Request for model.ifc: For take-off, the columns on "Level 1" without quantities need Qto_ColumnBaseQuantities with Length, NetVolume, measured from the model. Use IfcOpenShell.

First a look at what the model holds.

```python
import ifcopenshell
import ifcopenshell.util.element
import ifcopenshell.util.unit

model = ifcopenshell.open("model.ifc")
print(model.schema)
for unit_type in ("LENGTHUNIT", "AREAUNIT", "VOLUMEUNIT"):
    print(unit_type, ifcopenshell.util.unit.calculate_unit_scale(model, unit_type))
storey = next(s for s in model.by_type("IfcBuildingStorey") if s.Name == "Level 1")
columns = [e for e in ifcopenshell.util.element.get_decomposition(storey) if e.is_a("IfcColumn")]
for e in sorted(columns, key=lambda e: e.id()):
    print(e.id(), e.is_a(), e.Name, list(ifcopenshell.util.element.get_psets(e, qtos_only=True)), sep=" | ")
```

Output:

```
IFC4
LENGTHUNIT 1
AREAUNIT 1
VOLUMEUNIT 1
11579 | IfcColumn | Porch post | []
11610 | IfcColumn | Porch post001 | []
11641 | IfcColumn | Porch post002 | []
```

```python
import ifcopenshell
import ifcopenshell.api.pset
import ifcopenshell.geom
import ifcopenshell.util.element
import ifcopenshell.util.shape
import ifcopenshell.util.unit

model = ifcopenshell.open("model.ifc")
unit_scale = ifcopenshell.util.unit.calculate_unit_scale(model)
volume_scale = ifcopenshell.util.unit.calculate_unit_scale(model, "VOLUMEUNIT")
settings = ifcopenshell.geom.settings()

storey = next(s for s in model.by_type("IfcBuildingStorey") if s.Name == "Level 1")
columns = [e for e in ifcopenshell.util.element.get_decomposition(storey) if e.is_a("IfcColumn")]

for e in sorted(columns, key=lambda e: e.id()):
    if ifcopenshell.util.element.get_psets(e, qtos_only=True, should_inherit=False):
        continue
    # Geometry comes back in metres, in the element's own axes.
    shape = ifcopenshell.geom.create_shape(settings, e)
    values = {
        "Length": ifcopenshell.util.shape.get_z(shape.geometry) / unit_scale,
        "NetVolume": ifcopenshell.util.shape.get_volume(shape.geometry) / volume_scale,
    }
    qto = ifcopenshell.api.pset.add_qto(model, product=e, name="Qto_ColumnBaseQuantities")
    ifcopenshell.api.pset.edit_qto(model, qto=qto, properties=values)
    print(e.id(), {k: round(v, 3) for k, v in values.items()})

model.write("model_v2.ifc")
```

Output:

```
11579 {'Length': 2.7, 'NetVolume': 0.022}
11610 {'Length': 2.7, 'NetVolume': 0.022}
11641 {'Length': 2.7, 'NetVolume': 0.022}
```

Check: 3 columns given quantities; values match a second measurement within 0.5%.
